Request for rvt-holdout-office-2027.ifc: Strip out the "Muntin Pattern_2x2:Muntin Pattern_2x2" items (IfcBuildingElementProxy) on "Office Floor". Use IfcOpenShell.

First a look at what the model holds.

```python
import ifcopenshell
import ifcopenshell.util.element

model = ifcopenshell.open("rvt-holdout-office-2027.ifc")
print(model.schema)
storey = next(s for s in model.by_type("IfcBuildingStorey") if s.Name == "Office Floor")
proxies = [e for e in ifcopenshell.util.element.get_decomposition(storey) if e.is_a("IfcBuildingElementProxy")]
seen = {}
for e in proxies:
    element_type = ifcopenshell.util.element.get_type(e)
    name = element_type.Name if element_type not in (None, e) else None
    seen[name] = seen.get(name, 0) + 1
for name, count in sorted(seen.items(), key=str):
    print(count, "x", name)
```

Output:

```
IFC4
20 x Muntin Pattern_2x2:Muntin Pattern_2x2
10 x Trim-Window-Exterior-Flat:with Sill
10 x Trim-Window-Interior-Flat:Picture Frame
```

```python
import ifcopenshell
import ifcopenshell.api.root
import ifcopenshell.util.element

model = ifcopenshell.open("rvt-holdout-office-2027.ifc")

storey = next(s for s in model.by_type("IfcBuildingStorey") if s.Name == "Office Floor")
proxies = [e for e in ifcopenshell.util.element.get_decomposition(storey) if e.is_a("IfcBuildingElementProxy")]
targets = [e for e in proxies if (t := ifcopenshell.util.element.get_type(e)) not in (None, e) and t.Name == "Muntin Pattern_2x2:Muntin Pattern_2x2"]

for e in targets:
    ifcopenshell.api.root.remove_product(model, product=e)
print(len(targets), "removed")

model.write("rvt-holdout-office-2027_edited.ifc")
```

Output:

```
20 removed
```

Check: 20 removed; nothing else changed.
